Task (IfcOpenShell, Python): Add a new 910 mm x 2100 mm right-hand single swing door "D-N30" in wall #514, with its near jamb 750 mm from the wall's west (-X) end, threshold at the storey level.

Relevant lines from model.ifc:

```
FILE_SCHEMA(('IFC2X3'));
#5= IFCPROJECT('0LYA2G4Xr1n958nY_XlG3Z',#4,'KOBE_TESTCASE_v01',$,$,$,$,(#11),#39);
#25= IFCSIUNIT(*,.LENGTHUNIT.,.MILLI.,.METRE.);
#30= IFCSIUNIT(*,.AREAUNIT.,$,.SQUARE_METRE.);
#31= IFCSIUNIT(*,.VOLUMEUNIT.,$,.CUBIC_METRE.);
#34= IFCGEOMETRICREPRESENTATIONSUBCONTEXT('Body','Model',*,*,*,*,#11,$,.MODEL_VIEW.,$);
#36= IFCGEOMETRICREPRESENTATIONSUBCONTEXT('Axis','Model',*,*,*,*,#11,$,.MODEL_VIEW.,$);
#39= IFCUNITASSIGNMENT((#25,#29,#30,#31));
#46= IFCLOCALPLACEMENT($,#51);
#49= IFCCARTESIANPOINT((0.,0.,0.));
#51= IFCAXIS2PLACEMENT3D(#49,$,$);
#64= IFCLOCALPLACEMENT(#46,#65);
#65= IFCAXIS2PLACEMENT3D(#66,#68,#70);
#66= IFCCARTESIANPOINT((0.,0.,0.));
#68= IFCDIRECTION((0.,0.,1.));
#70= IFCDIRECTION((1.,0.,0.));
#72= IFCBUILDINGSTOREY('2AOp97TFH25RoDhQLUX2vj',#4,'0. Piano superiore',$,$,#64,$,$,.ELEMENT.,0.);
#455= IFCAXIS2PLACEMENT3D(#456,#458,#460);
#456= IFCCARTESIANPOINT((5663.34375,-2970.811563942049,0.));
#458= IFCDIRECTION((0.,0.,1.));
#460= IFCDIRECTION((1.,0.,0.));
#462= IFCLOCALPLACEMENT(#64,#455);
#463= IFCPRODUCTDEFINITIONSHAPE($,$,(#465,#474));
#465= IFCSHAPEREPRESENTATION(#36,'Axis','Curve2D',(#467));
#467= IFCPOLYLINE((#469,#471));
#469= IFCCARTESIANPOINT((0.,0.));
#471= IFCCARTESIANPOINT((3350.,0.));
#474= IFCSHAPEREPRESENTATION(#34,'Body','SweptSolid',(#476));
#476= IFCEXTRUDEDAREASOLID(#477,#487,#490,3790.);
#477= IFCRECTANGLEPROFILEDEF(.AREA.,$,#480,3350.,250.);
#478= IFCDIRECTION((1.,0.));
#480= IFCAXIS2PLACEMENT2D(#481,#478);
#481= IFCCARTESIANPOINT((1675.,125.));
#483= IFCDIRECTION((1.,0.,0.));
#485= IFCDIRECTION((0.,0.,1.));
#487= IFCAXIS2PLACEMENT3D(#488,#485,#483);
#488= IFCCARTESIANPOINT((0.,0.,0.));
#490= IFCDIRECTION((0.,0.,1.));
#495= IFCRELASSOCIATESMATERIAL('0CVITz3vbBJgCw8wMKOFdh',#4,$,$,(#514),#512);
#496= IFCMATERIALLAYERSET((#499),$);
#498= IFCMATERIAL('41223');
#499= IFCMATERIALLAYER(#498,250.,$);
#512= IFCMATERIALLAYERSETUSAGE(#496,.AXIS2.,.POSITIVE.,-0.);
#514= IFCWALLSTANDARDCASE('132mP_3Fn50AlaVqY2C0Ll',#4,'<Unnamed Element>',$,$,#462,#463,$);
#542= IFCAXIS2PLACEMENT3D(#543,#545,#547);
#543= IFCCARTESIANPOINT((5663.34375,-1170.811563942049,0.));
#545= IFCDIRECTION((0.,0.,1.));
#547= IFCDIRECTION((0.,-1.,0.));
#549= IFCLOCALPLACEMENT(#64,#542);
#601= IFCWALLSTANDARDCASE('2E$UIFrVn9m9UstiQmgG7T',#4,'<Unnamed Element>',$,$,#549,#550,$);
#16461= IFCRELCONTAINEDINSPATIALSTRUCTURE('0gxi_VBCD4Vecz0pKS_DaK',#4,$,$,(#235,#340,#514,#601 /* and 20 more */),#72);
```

```python
import numpy as np
import ifcopenshell
import ifcopenshell.api.feature
import ifcopenshell.api.geometry
import ifcopenshell.api.root
import ifcopenshell.api.spatial
import ifcopenshell.api.type
import ifcopenshell.geom
import ifcopenshell.util.element
import ifcopenshell.util.placement
import ifcopenshell.util.representation
import ifcopenshell.util.shape
import ifcopenshell.util.unit

model = ifcopenshell.open("model.ifc")
unit_scale = ifcopenshell.util.unit.calculate_unit_scale(model)
settings = ifcopenshell.geom.settings()


def volume(element):
    """Net volume in cubic metres, openings subtracted."""
    shape = ifcopenshell.geom.create_shape(settings, element)
    return ifcopenshell.util.shape.get_volume(shape.geometry)


wall = model.by_id(514)
storey = ifcopenshell.util.element.get_container(wall, ifc_class="IfcBuildingStorey")
context = ifcopenshell.util.representation.get_context(model, "Model", "Body", "MODEL_VIEW")
before = volume(wall)

width, height, from_end, sill = 0.91, 2.1, 0.75, 0.0  # metres

# The wall runs along its own X axis, and the end named is its -X end.
wall_shape = ifcopenshell.geom.create_shape(settings, wall)
x, y, z = ifcopenshell.util.shape.get_vertices(wall_shape.geometry).T
start = x.min() + from_end
face, thickness = float(y.min()), float(y.max() - y.min())
wall_matrix = ifcopenshell.util.placement.get_local_placement(wall.ObjectPlacement)
level = ifcopenshell.util.placement.get_local_placement(storey.ObjectPlacement)[2, 3]


def in_wall(x, y):
    """Placement at x, y metres in the wall's axes, at sill height."""
    matrix = wall_matrix.copy()
    matrix[:, 3] = wall_matrix @ np.array([x / unit_scale, y / unit_scale, 0.0, 1.0])
    matrix[2, 3] = level + sill / unit_scale
    return matrix


# Opening: a box that overshoots both wall faces by 50 mm.
opening = ifcopenshell.api.root.create_entity(model, ifc_class="IfcOpeningElement")
box = ifcopenshell.api.geometry.add_wall_representation(
    model, context=context, length=width, height=height, thickness=thickness + 0.1
)
ifcopenshell.api.geometry.assign_representation(model, product=opening, representation=box)
ifcopenshell.api.geometry.edit_object_placement(model, product=opening, matrix=in_wall(start, face - 0.05), is_si=False)
ifcopenshell.api.feature.add_feature(model, feature=opening, element=wall)

door = ifcopenshell.api.root.create_entity(model, ifc_class="IfcDoor", name="D-N30")
door.OverallWidth, door.OverallHeight = width / unit_scale, height / unit_scale
body = ifcopenshell.api.geometry.add_door_representation(
    model,
    context=context,
    overall_width=door.OverallWidth,
    overall_height=door.OverallHeight,
    operation_type="SINGLE_SWING_RIGHT",
    lining_properties={"LiningDepth": thickness / unit_scale, "ThresholdDepth": thickness / unit_scale},
)
ifcopenshell.api.geometry.assign_representation(model, product=door, representation=body)
ifcopenshell.api.spatial.assign_container(model, products=[door], relating_structure=storey)
fills = ifcopenshell.api.feature.add_filling(model, opening=opening, element=door)
fills.OwnerHistory = door.OwnerHistory  # required in IFC2X3

# IFC2X3 keeps the operation on the door style.
style = ifcopenshell.api.root.create_entity(model, ifc_class="IfcDoorStyle", name="D-N30")
style.OperationType, style.ConstructionType = "SINGLE_SWING_RIGHT", "NOTDEFINED"
style.ParameterTakesPrecedence = style.Sizeable = False
ifcopenshell.api.type.assign_type(model, related_objects=[door], relating_type=style)

# The lining spans the wall, so the door starts at the wall face.
ifcopenshell.api.geometry.edit_object_placement(model, product=door, matrix=in_wall(start, face), is_si=False)

after = volume(wall)

print(f"wall volume {before:.3f} -> {after:.3f} m3")

model.write("model_v2.ifc")
```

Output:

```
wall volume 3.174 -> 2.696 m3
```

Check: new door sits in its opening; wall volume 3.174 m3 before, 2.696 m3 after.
